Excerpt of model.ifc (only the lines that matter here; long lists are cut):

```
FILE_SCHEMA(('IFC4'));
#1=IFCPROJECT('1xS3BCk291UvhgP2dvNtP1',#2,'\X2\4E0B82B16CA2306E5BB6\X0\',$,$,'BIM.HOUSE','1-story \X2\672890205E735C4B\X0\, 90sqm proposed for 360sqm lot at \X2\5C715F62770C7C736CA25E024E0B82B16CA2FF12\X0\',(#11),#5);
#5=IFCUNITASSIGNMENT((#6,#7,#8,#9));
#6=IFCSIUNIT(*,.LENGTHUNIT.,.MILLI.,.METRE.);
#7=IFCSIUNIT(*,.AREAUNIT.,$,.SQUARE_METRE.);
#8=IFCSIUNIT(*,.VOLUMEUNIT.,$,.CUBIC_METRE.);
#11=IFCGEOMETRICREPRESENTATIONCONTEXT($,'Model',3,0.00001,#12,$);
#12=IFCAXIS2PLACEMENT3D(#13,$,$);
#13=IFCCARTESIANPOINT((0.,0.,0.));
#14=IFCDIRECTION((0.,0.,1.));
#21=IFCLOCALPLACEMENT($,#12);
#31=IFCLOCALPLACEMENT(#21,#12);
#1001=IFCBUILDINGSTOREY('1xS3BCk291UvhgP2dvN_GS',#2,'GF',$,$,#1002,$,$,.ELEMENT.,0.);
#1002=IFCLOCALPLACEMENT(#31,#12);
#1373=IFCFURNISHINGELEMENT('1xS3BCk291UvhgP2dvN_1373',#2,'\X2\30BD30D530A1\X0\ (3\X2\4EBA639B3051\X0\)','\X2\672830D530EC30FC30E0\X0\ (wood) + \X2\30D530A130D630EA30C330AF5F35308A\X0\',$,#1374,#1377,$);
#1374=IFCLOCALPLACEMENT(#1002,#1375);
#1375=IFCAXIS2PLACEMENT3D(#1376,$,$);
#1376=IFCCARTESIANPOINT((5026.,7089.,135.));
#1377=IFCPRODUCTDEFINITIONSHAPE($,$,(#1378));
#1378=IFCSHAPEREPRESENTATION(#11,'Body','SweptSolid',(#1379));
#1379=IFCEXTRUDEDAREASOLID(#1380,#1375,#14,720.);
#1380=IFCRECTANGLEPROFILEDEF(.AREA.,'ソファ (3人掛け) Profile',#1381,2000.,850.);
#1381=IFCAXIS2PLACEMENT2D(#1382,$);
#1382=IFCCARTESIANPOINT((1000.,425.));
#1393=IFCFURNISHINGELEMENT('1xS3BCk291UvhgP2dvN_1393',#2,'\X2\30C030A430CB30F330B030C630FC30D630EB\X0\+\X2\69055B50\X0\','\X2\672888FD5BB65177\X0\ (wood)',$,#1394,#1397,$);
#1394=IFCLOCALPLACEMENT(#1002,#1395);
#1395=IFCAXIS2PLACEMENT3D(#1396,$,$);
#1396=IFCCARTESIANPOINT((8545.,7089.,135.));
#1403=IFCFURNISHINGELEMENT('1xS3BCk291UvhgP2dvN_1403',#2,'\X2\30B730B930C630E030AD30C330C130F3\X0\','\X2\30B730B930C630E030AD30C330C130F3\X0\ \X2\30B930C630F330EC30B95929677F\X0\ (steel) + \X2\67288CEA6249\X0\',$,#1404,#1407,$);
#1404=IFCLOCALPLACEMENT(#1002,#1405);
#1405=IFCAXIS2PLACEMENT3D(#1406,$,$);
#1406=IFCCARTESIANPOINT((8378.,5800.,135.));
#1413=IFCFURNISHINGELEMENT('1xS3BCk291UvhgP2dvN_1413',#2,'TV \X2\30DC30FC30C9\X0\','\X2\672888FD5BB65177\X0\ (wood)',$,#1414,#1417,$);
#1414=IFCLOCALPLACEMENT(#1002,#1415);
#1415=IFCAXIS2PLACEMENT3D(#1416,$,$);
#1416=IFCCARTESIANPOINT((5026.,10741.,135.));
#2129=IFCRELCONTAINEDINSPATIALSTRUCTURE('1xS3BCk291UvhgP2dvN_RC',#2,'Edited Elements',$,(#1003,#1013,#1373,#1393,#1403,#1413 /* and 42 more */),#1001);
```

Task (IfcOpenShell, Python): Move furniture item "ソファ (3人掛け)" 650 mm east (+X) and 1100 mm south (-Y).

```python
import ifcopenshell
import ifcopenshell.api.geometry
import ifcopenshell.util.placement
import ifcopenshell.util.unit

model = ifcopenshell.open("model.ifc")
unit_scale = ifcopenshell.util.unit.calculate_unit_scale(model)

item = model.by_guid("1xS3BCk291UvhgP2dvN_1373")
matrix = ifcopenshell.util.placement.get_local_placement(item.ObjectPlacement)
matrix[0, 3] += 0.65 / unit_scale
matrix[1, 3] -= 1.1 / unit_scale
ifcopenshell.api.geometry.edit_object_placement(model, product=item, matrix=matrix, is_si=False)

print(ifcopenshell.util.placement.get_local_placement(item.ObjectPlacement).round(3) + 0.0)

model.write("model_rev.ifc")
```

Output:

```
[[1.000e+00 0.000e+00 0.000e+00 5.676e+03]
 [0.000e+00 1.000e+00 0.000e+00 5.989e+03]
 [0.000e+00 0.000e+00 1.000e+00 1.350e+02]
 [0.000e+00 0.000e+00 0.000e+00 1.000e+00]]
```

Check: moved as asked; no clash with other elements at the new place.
